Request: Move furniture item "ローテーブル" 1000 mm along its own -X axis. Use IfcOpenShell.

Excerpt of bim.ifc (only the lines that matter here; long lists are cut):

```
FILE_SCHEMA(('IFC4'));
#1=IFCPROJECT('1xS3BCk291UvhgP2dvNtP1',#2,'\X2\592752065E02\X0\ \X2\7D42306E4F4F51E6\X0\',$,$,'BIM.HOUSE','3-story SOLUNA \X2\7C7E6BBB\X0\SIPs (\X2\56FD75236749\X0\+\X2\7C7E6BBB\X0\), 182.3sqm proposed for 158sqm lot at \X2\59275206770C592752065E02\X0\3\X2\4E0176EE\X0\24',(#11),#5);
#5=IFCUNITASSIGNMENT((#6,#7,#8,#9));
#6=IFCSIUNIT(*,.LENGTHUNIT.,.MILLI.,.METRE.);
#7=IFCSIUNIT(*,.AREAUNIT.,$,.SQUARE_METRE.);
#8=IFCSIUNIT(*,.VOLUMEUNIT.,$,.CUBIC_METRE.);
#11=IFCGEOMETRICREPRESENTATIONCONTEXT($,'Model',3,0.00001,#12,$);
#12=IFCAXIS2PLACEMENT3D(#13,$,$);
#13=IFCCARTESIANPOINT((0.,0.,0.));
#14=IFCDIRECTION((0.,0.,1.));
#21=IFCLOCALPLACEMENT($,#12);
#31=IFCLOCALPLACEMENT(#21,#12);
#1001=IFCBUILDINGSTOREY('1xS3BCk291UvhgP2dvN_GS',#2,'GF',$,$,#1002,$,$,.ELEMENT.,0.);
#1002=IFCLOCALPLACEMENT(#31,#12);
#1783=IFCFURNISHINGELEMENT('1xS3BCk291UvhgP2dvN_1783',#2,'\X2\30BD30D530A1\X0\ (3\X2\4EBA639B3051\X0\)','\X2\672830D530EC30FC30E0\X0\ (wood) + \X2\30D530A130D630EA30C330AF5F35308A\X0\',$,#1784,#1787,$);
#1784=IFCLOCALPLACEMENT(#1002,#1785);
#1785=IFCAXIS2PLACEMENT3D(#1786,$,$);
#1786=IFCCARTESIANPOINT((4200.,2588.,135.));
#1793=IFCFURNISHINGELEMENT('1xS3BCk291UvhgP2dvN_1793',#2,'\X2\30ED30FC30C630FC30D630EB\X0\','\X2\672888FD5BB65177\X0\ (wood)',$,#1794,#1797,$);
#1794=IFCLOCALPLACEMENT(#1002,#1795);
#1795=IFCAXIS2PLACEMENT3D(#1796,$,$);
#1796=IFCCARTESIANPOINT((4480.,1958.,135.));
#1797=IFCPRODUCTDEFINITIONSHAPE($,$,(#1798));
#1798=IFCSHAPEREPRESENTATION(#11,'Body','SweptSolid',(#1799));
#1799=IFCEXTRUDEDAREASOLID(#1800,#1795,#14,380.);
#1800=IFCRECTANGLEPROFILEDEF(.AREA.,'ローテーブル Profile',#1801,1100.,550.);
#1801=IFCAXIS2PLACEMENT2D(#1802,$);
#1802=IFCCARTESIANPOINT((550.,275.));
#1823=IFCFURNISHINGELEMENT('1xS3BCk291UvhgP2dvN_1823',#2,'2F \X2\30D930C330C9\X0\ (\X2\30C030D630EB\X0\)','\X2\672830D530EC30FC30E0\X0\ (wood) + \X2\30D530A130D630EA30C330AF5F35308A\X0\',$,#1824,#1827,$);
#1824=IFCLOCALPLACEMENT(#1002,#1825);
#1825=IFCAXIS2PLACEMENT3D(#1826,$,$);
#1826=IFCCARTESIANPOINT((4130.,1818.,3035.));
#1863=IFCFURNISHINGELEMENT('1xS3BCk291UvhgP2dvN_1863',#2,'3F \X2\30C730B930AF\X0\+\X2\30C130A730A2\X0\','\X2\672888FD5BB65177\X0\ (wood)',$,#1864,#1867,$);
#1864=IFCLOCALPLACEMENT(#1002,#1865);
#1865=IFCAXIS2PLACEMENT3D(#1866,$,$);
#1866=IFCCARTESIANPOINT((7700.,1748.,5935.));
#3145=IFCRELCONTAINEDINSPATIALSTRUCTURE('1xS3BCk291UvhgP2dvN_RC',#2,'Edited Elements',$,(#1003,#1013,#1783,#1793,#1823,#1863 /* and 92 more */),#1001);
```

```python
import ifcopenshell
import ifcopenshell.api.geometry
import ifcopenshell.util.placement

model = ifcopenshell.open("bim.ifc")

item = model.by_id(1793)
matrix = ifcopenshell.util.placement.get_local_placement(item.ObjectPlacement)
matrix[:3, 3] -= matrix[:3, 0] * 1000.0
ifcopenshell.api.geometry.edit_object_placement(model, product=item, matrix=matrix, is_si=False)

print(ifcopenshell.util.placement.get_local_placement(item.ObjectPlacement).round(3) + 0.0)

model.write("bim_v2.ifc")
```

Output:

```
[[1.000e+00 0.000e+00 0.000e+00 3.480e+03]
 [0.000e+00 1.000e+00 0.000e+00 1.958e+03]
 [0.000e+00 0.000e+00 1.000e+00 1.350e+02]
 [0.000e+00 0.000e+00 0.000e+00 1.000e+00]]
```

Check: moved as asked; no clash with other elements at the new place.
